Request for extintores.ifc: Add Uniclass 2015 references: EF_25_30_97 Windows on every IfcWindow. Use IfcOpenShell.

First a look at what the model holds.

```python
import ifcopenshell

model = ifcopenshell.open("extintores.ifc")
print(model.schema)
print("classifications:", [c.Name for c in model.by_type("IfcClassification")])
for ifc_class in ("IfcDoor", "IfcRoof", "IfcStair", "IfcWall", "IfcWindow"):
    print(ifc_class, len(model.by_type(ifc_class)))
```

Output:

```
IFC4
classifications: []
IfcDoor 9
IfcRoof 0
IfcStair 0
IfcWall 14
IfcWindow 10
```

```python
import ifcopenshell
import ifcopenshell.api.classification

model = ifcopenshell.open("extintores.ifc")

system = ifcopenshell.api.classification.add_classification(model, classification="Uniclass 2015")

codes = {
    "IfcWindow": ("EF_25_30_97", "Windows"),
}
for ifc_class, (code, name) in codes.items():
    products = model.by_type(ifc_class)
    ifcopenshell.api.classification.add_reference(
        model, products=products, classification=system, identification=code, name=name
    )
    print(code, len(products))

model.write("extintores_updated.ifc")
```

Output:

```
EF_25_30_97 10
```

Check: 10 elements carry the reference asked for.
